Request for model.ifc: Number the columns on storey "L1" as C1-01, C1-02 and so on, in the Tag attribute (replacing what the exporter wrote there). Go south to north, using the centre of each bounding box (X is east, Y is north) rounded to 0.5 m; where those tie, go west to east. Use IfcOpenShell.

First a look at what the model holds.

```python
import ifcopenshell
import ifcopenshell.util.element
import ifcopenshell.util.placement

model = ifcopenshell.open("model.ifc")
print(model.schema)
storey = next(s for s in model.by_type("IfcBuildingStorey") if s.Name == "L1")
columns = [e for e in ifcopenshell.util.element.get_decomposition(storey) if e.is_a("IfcColumn")]
for e in sorted(columns, key=lambda e: e.id()):
    origin = ifcopenshell.util.placement.get_local_placement(e.ObjectPlacement)[:3, 3]
    print(e.id(), e.Tag, e.Name, origin.round(2) + 0.0, sep=" | ")
```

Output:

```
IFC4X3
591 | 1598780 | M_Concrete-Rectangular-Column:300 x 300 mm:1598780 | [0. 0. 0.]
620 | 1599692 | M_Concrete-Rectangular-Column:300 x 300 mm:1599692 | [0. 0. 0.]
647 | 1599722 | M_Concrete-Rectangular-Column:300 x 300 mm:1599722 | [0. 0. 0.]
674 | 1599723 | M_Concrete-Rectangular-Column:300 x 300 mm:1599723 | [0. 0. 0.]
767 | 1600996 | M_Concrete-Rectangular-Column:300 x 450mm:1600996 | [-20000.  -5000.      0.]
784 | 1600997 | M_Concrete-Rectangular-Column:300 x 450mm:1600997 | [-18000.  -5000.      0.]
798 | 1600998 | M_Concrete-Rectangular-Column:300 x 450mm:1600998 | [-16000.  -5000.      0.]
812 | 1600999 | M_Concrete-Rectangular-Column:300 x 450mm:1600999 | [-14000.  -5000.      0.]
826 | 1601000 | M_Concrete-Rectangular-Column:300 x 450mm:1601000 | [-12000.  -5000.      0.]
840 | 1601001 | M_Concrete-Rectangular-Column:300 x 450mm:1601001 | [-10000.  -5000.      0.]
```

```python
import ifcopenshell
import ifcopenshell.geom
import ifcopenshell.util.element
import ifcopenshell.util.shape

model = ifcopenshell.open("model.ifc")
settings = ifcopenshell.geom.settings()
settings.set("use-world-coords", True)


def centre(element):
    shape = ifcopenshell.geom.create_shape(settings, element)
    return ifcopenshell.util.shape.get_bbox_centroid(shape.geometry)


storey = next(s for s in model.by_type("IfcBuildingStorey") if s.Name == "L1")
columns = [e for e in ifcopenshell.util.element.get_decomposition(storey) if e.is_a("IfcColumn")]

# Insertion points can sit at a corner or the storey origin, so sort by the geometry (in metres).
centres = {e: centre(e) for e in columns}
columns.sort(key=lambda e: (round(centres[e][1] / 0.5), centres[e][0]))

for i, e in enumerate(columns, start=1):
    number = f"C1-{i:02d}"
    e.Tag = number
    print(e.id(), number)

model.write("model_edited.ifc")
```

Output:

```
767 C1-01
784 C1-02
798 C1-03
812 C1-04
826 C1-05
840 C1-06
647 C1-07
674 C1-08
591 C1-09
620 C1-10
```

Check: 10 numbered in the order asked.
